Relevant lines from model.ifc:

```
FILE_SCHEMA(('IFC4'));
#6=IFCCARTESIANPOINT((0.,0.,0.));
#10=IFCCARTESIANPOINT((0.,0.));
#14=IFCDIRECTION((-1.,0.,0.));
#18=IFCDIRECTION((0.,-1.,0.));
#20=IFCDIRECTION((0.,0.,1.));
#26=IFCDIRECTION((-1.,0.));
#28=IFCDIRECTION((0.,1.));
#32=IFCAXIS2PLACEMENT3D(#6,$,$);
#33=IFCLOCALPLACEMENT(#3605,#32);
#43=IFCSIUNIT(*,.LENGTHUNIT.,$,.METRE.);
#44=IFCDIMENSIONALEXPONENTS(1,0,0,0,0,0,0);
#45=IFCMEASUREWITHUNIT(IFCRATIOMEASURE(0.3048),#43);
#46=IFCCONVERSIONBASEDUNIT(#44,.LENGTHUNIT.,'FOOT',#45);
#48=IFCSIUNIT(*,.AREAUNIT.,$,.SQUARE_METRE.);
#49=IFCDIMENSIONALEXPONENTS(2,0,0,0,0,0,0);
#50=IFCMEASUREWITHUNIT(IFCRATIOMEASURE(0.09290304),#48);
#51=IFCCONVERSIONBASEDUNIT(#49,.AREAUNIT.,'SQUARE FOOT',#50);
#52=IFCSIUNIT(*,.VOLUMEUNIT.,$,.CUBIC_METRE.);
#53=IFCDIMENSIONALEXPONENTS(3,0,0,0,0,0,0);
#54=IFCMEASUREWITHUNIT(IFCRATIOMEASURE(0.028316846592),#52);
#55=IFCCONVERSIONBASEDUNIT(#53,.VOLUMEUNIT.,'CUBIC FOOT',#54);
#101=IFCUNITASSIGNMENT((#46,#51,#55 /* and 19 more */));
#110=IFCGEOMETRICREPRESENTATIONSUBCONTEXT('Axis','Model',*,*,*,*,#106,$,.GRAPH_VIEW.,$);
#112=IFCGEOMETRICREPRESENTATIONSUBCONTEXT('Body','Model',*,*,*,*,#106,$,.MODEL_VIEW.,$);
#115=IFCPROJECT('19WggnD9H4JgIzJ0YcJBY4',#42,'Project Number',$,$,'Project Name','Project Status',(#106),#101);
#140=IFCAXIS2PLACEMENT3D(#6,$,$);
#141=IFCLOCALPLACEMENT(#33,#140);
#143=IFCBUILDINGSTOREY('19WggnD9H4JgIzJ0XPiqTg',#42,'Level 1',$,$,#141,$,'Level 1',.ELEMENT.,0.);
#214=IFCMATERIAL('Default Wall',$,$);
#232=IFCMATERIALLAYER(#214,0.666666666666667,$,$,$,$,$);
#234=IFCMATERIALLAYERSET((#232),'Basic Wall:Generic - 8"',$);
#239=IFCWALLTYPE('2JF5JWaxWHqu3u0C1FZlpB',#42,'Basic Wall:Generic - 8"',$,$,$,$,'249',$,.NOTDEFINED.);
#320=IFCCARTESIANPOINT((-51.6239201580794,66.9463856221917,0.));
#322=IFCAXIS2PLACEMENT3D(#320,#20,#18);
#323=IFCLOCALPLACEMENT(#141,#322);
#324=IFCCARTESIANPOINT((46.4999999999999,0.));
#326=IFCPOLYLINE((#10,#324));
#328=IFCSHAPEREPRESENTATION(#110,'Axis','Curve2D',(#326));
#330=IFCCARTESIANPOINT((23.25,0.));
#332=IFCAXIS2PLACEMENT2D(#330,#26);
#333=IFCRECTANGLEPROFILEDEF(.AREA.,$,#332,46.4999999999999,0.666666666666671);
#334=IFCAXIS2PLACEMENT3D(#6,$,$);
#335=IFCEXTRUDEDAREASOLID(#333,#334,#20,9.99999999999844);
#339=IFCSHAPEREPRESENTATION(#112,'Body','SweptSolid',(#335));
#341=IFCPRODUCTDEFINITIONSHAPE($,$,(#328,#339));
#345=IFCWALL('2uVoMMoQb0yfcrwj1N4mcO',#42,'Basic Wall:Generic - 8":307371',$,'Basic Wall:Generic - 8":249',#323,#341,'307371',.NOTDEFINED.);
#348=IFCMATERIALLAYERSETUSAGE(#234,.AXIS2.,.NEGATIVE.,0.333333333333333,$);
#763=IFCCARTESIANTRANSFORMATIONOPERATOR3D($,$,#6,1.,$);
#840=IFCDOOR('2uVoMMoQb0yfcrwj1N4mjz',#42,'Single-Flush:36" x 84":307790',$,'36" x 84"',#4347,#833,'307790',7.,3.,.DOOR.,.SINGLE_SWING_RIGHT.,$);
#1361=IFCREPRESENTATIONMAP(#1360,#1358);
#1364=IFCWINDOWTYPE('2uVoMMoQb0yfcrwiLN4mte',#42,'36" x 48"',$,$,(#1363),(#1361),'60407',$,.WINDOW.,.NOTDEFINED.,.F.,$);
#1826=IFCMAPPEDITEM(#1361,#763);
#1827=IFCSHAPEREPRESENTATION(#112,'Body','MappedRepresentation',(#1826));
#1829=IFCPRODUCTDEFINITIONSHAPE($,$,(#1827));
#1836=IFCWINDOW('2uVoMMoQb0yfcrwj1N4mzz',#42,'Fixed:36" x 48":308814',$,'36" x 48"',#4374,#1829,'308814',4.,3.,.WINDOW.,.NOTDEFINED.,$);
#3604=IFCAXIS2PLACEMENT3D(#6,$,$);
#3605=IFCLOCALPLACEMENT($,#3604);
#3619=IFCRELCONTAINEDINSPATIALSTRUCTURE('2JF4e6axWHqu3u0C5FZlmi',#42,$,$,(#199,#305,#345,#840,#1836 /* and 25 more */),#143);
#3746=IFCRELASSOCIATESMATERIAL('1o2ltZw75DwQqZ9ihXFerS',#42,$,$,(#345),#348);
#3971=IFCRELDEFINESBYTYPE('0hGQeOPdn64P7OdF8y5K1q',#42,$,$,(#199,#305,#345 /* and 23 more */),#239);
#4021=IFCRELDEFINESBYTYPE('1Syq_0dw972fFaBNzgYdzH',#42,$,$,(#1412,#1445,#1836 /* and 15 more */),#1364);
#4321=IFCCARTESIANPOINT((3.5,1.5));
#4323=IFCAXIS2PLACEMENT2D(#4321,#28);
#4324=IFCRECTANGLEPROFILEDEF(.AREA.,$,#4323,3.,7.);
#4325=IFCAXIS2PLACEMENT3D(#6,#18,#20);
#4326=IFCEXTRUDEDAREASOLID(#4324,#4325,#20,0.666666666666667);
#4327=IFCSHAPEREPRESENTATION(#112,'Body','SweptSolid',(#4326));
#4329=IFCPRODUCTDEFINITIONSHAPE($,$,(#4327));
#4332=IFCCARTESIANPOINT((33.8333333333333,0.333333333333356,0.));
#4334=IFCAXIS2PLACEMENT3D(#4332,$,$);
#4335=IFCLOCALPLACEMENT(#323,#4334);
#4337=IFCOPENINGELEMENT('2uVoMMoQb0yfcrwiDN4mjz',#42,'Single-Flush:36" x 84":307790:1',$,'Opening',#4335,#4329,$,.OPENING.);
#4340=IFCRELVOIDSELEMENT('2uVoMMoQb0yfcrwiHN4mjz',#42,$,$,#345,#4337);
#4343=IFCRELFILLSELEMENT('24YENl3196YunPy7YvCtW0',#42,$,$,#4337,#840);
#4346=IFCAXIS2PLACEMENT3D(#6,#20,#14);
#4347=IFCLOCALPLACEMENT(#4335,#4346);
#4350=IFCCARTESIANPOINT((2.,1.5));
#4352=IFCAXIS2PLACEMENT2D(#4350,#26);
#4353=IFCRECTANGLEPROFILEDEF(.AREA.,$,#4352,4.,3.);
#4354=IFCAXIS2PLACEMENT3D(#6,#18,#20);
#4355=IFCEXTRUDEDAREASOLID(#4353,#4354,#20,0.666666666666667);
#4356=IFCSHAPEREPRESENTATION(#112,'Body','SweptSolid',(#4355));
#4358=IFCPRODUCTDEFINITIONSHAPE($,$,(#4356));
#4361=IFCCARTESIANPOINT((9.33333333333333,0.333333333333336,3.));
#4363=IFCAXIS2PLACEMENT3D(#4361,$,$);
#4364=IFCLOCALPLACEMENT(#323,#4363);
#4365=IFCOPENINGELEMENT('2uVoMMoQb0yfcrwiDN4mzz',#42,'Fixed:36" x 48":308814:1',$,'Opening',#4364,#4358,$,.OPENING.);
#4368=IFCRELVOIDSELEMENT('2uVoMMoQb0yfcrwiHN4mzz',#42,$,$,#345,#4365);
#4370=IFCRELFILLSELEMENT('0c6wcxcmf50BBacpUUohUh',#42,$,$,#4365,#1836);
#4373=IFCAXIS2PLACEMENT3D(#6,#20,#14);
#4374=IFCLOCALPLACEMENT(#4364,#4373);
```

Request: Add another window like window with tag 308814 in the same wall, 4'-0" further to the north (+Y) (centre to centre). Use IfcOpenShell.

```python
import ifcopenshell
import ifcopenshell.api.feature
import ifcopenshell.api.geometry
import ifcopenshell.api.root
import ifcopenshell.geom
import ifcopenshell.util.element
import ifcopenshell.util.placement
import ifcopenshell.util.shape
import ifcopenshell.util.unit

model = ifcopenshell.open("model.ifc")
unit_scale = ifcopenshell.util.unit.calculate_unit_scale(model)
settings = ifcopenshell.geom.settings()


def volume(element):
    """Net volume in cubic metres, openings subtracted."""
    shape = ifcopenshell.geom.create_shape(settings, element)
    return ifcopenshell.util.shape.get_volume(shape.geometry)


def reuse_history(source, copy):
    """copy_class also copies each property set's owner history, people and application; keep the originals."""
    for rel in copy.IsDefinedBy:
        if rel.is_a("IfcRelDefinesByProperties") and (history := rel.RelatingPropertyDefinition.OwnerHistory):
            rel.RelatingPropertyDefinition.OwnerHistory = source.OwnerHistory
            ifcopenshell.util.element.remove_deep2(model, history)


window = model.by_id(1836)
opening = window.FillsVoids[0].RelatingOpeningElement
wall = opening.VoidsElements[0].RelatingBuildingElement
before = volume(wall)
shift = ifcopenshell.util.placement.get_local_placement(wall.ObjectPlacement)[:3, 0] * -48 * 0.0254 / unit_scale

# copy_class copies the void relationship, type, container and properties, but no geometry.
new_opening = ifcopenshell.api.root.copy_class(model, product=opening)
new_opening.Representation = ifcopenshell.util.element.copy_deep(
    model, opening.Representation, exclude=["IfcGeometricRepresentationContext", "IfcRepresentationMap"]
)
new_opening.Name = 'Fixed:36" x 48"'
new_window = ifcopenshell.api.root.copy_class(model, product=window)
new_window.Representation = ifcopenshell.util.element.copy_deep(
    model, window.Representation, exclude=["IfcGeometricRepresentationContext", "IfcRepresentationMap"]
)
new_window.Name = 'Fixed:36" x 48"'
new_window.Tag = None
reuse_history(window, new_window)
ifcopenshell.api.feature.add_filling(model, opening=new_opening, element=new_window)

for old, new in ((opening, new_opening), (window, new_window)):
    matrix = ifcopenshell.util.placement.get_local_placement(old.ObjectPlacement)
    matrix[:3, 3] += shift
    ifcopenshell.api.geometry.edit_object_placement(model, product=new, matrix=matrix, is_si=False)

after = volume(wall)

print(f"wall volume {before:.3f} -> {after:.3f} m3")

model.write("model_updated.ifc")
```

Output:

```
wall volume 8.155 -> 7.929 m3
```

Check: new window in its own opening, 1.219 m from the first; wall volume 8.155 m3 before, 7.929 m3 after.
